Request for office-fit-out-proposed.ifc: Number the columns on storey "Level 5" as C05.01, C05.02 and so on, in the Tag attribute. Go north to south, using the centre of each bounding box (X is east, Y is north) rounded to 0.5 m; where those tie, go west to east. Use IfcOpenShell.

First a look at what the model holds.

```python
import ifcopenshell
import ifcopenshell.util.element
import ifcopenshell.util.placement

model = ifcopenshell.open("office-fit-out-proposed.ifc")
print(model.schema)
storey = next(s for s in model.by_type("IfcBuildingStorey") if s.Name == "Level 5")
columns = [e for e in ifcopenshell.util.element.get_decomposition(storey) if e.is_a("IfcColumn")]
for e in sorted(columns, key=lambda e: e.id()):
    origin = ifcopenshell.util.placement.get_local_placement(e.ObjectPlacement)[:3, 3]
    print(e.id(), e.Tag, e.Name, origin.round(2) + 0.0, sep=" | ")
```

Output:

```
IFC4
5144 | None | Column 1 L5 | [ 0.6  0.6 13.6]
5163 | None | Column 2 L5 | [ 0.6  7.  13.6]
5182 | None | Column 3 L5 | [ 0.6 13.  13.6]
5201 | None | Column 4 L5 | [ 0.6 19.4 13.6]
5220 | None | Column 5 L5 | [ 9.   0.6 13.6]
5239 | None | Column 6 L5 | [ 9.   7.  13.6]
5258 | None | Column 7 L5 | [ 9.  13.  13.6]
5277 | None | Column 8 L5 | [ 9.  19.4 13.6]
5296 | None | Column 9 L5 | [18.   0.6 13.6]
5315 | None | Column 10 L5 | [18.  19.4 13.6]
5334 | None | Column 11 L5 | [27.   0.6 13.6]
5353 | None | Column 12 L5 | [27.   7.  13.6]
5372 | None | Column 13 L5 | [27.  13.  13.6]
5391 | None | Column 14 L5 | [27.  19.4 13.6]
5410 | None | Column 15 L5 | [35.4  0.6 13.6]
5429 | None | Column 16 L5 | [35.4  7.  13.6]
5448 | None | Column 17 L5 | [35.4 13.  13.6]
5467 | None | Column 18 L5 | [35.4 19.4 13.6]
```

```python
import ifcopenshell
import ifcopenshell.geom
import ifcopenshell.util.element
import ifcopenshell.util.shape

model = ifcopenshell.open("office-fit-out-proposed.ifc")
settings = ifcopenshell.geom.settings()
settings.set("use-world-coords", True)


def centre(element):
    shape = ifcopenshell.geom.create_shape(settings, element)
    return ifcopenshell.util.shape.get_bbox_centroid(shape.geometry)


storey = next(s for s in model.by_type("IfcBuildingStorey") if s.Name == "Level 5")
columns = [e for e in ifcopenshell.util.element.get_decomposition(storey) if e.is_a("IfcColumn")]

# Insertion points can sit at a corner or the storey origin, so sort by the geometry (in metres).
centres = {e: centre(e) for e in columns}
columns.sort(key=lambda e: (-round(centres[e][1] / 0.5), centres[e][0]))

for i, e in enumerate(columns, start=1):
    number = f"C05.{i:02d}"
    e.Tag = number
    print(e.id(), number)

model.write("office-fit-out-proposed_rev.ifc")
```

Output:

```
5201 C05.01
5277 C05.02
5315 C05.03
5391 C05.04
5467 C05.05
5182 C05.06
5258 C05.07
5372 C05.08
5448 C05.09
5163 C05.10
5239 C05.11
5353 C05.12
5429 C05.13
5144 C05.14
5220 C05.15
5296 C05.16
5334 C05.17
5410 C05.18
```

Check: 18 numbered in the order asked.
